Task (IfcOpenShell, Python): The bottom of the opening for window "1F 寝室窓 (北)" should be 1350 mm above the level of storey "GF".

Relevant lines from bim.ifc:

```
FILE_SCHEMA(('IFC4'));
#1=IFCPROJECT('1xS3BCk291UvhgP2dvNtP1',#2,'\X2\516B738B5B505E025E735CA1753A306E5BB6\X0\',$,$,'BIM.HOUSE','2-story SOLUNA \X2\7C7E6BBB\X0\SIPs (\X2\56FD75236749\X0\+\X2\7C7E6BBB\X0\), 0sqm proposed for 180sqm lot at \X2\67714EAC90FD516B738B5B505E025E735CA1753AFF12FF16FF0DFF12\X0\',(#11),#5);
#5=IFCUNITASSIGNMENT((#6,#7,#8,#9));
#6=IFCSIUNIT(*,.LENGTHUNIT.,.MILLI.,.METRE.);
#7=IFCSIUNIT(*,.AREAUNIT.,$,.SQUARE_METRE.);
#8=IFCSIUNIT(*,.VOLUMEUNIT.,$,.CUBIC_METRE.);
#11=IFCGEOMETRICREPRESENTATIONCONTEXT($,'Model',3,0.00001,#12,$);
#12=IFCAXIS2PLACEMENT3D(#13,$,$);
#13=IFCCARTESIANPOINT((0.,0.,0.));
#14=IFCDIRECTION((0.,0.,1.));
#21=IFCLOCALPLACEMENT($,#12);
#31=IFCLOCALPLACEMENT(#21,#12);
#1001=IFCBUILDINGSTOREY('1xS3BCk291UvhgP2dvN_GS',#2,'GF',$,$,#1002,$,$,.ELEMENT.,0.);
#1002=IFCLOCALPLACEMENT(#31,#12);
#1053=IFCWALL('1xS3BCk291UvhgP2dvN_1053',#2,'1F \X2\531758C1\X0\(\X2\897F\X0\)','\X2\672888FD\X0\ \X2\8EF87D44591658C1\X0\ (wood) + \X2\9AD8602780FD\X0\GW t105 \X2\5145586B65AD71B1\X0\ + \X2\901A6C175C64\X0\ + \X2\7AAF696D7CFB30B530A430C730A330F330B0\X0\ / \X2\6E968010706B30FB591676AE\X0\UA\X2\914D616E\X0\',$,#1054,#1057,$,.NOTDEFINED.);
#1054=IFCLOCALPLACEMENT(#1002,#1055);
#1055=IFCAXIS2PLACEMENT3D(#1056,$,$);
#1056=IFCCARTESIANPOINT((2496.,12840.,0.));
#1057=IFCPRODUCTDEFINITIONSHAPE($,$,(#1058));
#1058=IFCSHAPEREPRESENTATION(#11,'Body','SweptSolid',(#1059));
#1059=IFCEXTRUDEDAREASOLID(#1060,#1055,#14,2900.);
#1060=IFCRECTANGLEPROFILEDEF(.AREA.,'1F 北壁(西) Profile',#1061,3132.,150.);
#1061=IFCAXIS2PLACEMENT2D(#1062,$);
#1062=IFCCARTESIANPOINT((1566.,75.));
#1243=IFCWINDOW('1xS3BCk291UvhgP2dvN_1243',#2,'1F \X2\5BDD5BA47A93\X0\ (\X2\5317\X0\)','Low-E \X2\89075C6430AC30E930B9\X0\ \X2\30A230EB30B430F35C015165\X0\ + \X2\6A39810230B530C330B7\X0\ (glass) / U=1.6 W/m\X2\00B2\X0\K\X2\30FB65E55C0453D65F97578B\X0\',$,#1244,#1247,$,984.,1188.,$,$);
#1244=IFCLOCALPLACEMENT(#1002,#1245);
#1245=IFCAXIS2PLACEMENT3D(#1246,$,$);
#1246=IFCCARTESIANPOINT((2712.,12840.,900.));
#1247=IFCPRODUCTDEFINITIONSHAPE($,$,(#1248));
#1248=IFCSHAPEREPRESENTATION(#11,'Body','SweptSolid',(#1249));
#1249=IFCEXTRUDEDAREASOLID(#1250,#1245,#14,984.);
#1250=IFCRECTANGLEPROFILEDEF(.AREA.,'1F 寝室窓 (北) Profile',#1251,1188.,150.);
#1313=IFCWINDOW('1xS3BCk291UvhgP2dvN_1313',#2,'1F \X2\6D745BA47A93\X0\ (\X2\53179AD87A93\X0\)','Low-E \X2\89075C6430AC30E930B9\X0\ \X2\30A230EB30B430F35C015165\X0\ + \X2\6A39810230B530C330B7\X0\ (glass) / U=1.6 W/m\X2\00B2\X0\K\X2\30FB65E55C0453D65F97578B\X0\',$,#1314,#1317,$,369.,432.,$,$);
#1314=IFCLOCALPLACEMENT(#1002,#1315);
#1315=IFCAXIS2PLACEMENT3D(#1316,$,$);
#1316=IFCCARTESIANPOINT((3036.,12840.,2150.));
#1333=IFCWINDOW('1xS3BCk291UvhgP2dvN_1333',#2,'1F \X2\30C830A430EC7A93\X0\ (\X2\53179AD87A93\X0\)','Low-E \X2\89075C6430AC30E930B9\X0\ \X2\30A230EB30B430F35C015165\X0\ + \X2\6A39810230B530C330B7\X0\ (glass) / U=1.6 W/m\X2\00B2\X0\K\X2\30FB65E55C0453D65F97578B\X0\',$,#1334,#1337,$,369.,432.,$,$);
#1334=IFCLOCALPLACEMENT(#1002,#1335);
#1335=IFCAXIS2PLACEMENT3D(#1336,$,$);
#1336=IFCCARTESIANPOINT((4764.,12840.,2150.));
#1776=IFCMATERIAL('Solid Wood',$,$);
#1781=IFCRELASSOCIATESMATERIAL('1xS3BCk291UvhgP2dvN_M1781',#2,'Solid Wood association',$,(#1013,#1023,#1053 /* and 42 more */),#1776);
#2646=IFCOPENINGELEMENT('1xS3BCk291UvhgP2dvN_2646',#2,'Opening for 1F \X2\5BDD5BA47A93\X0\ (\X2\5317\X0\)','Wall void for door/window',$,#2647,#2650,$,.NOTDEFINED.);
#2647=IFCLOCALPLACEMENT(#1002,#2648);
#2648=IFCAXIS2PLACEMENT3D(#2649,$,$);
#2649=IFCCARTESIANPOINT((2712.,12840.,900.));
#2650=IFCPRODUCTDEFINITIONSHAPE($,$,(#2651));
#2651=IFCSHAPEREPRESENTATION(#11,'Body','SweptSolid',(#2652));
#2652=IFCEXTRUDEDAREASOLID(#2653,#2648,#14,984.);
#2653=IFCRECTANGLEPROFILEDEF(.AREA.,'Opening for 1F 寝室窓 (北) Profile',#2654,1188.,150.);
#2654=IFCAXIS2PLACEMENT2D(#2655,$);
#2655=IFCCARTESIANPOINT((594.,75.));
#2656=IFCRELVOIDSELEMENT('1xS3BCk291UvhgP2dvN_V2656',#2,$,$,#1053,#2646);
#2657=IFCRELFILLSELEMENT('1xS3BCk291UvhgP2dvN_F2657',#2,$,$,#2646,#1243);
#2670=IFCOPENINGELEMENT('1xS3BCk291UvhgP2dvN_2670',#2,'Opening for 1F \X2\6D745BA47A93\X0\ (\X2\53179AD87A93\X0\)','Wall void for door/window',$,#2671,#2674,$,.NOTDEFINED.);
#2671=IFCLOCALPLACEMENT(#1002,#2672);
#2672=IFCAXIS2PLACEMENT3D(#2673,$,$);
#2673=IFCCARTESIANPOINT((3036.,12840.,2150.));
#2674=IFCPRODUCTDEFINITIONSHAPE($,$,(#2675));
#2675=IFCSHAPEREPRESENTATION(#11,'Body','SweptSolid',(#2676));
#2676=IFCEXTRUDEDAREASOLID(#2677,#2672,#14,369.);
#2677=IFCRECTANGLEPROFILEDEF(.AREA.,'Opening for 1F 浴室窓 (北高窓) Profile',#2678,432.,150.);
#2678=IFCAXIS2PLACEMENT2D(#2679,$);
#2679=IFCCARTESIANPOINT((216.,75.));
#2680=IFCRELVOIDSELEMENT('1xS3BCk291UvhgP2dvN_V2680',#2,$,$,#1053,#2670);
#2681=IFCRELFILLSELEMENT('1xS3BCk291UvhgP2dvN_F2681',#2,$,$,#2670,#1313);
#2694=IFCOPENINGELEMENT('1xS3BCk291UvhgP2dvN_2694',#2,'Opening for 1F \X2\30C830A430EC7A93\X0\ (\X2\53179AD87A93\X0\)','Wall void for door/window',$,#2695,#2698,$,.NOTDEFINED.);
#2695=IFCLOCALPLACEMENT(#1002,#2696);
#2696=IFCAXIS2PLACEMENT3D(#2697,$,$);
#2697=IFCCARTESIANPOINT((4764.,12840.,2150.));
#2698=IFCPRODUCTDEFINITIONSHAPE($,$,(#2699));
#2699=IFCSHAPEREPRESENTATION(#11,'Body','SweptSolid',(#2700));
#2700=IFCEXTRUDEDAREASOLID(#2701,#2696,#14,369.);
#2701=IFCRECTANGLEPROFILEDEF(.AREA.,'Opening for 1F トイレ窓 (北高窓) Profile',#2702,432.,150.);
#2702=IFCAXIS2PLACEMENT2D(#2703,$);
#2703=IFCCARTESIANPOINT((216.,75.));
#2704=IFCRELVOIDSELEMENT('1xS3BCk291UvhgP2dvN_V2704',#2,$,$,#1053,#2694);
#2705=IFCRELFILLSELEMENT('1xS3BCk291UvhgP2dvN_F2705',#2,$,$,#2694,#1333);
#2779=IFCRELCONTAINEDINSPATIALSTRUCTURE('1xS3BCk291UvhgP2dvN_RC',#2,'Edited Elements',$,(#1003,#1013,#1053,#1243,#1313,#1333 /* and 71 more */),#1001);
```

```python
import numpy as np
import ifcopenshell
import ifcopenshell.api.geometry
import ifcopenshell.geom
import ifcopenshell.util.element
import ifcopenshell.util.placement
import ifcopenshell.util.shape
import ifcopenshell.util.unit

model = ifcopenshell.open("bim.ifc")
unit_scale = ifcopenshell.util.unit.calculate_unit_scale(model)

window = model.by_guid("1xS3BCk291UvhgP2dvN_1243")
opening = window.FillsVoids[0].RelatingOpeningElement
storey = ifcopenshell.util.element.get_container(window, ifc_class="IfcBuildingStorey")
level = ifcopenshell.util.placement.get_local_placement(storey.ObjectPlacement)[2, 3]

# The opening's origin need not be at the sill, so measure its lowest point.
shape = ifcopenshell.geom.create_shape(ifcopenshell.geom.settings(), opening)
bottom = ifcopenshell.util.shape.get_shape_bottom_elevation(shape, shape.geometry) / unit_scale
dz = level + 1350.0 - bottom

shift = np.array([0.0, 0.0, dz])
# The window is not placed relative to its opening, so move both.
for product in (opening, window):
    matrix = ifcopenshell.util.placement.get_local_placement(product.ObjectPlacement)
    matrix[:3, 3] += shift
    ifcopenshell.api.geometry.edit_object_placement(model, product=product, matrix=matrix, is_si=False)

print(f"moved by {dz * unit_scale:+.3f} m")

model.write("bim_rev.ifc")
```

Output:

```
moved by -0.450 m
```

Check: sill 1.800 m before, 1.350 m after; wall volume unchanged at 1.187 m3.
